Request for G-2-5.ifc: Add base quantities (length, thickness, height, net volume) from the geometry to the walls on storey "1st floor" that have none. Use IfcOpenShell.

First a look at what the model holds.

```python
import ifcopenshell
import ifcopenshell.util.element
import ifcopenshell.util.unit

model = ifcopenshell.open("G-2-5.ifc")
print(model.schema)
for unit_type in ("LENGTHUNIT", "AREAUNIT", "VOLUMEUNIT"):
    print(unit_type, ifcopenshell.util.unit.calculate_unit_scale(model, unit_type))
storey = next(s for s in model.by_type("IfcBuildingStorey") if s.Name == "1st floor")
walls = [e for e in ifcopenshell.util.element.get_decomposition(storey) if e.is_a("IfcWall")]
for e in sorted(walls, key=lambda e: e.id()):
    print(e.id(), e.is_a(), e.Name, list(ifcopenshell.util.element.get_psets(e, qtos_only=True)), sep=" | ")
```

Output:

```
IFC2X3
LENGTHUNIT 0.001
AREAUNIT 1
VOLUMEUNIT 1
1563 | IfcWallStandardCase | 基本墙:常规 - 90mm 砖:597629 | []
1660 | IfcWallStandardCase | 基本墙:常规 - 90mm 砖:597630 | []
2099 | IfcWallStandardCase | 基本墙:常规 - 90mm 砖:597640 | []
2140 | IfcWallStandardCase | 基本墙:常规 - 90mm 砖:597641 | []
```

```python
import ifcopenshell
import ifcopenshell.api.pset
import ifcopenshell.geom
import ifcopenshell.util.element
import ifcopenshell.util.shape
import ifcopenshell.util.unit

model = ifcopenshell.open("G-2-5.ifc")
unit_scale = ifcopenshell.util.unit.calculate_unit_scale(model)
volume_scale = ifcopenshell.util.unit.calculate_unit_scale(model, "VOLUMEUNIT")
settings = ifcopenshell.geom.settings()

storey = next(s for s in model.by_type("IfcBuildingStorey") if s.Name == "1st floor")
walls = [e for e in ifcopenshell.util.element.get_decomposition(storey) if e.is_a("IfcWall")]

for e in sorted(walls, key=lambda e: e.id()):
    if ifcopenshell.util.element.get_psets(e, qtos_only=True, should_inherit=False):
        continue
    # Geometry comes back in metres, in the element's own axes.
    shape = ifcopenshell.geom.create_shape(settings, e)
    values = {
        "Length": ifcopenshell.util.shape.get_x(shape.geometry) / unit_scale,
        "Width": ifcopenshell.util.shape.get_y(shape.geometry) / unit_scale,
        "Height": ifcopenshell.util.shape.get_z(shape.geometry) / unit_scale,
        "NetVolume": ifcopenshell.util.shape.get_volume(shape.geometry) / volume_scale,
    }
    qto = ifcopenshell.api.pset.add_qto(model, product=e, name="BaseQuantities")
    ifcopenshell.api.pset.edit_qto(model, qto=qto, properties=values)
    print(e.id(), {k: round(v, 3) for k, v in values.items()})

model.write("G-2-5_v2.ifc")
```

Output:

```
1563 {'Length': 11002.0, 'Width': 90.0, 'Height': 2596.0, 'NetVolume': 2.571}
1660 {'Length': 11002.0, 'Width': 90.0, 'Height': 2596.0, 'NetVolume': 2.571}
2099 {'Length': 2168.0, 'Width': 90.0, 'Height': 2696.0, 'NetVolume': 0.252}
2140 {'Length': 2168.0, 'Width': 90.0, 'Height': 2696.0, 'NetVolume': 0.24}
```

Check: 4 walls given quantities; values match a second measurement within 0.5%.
